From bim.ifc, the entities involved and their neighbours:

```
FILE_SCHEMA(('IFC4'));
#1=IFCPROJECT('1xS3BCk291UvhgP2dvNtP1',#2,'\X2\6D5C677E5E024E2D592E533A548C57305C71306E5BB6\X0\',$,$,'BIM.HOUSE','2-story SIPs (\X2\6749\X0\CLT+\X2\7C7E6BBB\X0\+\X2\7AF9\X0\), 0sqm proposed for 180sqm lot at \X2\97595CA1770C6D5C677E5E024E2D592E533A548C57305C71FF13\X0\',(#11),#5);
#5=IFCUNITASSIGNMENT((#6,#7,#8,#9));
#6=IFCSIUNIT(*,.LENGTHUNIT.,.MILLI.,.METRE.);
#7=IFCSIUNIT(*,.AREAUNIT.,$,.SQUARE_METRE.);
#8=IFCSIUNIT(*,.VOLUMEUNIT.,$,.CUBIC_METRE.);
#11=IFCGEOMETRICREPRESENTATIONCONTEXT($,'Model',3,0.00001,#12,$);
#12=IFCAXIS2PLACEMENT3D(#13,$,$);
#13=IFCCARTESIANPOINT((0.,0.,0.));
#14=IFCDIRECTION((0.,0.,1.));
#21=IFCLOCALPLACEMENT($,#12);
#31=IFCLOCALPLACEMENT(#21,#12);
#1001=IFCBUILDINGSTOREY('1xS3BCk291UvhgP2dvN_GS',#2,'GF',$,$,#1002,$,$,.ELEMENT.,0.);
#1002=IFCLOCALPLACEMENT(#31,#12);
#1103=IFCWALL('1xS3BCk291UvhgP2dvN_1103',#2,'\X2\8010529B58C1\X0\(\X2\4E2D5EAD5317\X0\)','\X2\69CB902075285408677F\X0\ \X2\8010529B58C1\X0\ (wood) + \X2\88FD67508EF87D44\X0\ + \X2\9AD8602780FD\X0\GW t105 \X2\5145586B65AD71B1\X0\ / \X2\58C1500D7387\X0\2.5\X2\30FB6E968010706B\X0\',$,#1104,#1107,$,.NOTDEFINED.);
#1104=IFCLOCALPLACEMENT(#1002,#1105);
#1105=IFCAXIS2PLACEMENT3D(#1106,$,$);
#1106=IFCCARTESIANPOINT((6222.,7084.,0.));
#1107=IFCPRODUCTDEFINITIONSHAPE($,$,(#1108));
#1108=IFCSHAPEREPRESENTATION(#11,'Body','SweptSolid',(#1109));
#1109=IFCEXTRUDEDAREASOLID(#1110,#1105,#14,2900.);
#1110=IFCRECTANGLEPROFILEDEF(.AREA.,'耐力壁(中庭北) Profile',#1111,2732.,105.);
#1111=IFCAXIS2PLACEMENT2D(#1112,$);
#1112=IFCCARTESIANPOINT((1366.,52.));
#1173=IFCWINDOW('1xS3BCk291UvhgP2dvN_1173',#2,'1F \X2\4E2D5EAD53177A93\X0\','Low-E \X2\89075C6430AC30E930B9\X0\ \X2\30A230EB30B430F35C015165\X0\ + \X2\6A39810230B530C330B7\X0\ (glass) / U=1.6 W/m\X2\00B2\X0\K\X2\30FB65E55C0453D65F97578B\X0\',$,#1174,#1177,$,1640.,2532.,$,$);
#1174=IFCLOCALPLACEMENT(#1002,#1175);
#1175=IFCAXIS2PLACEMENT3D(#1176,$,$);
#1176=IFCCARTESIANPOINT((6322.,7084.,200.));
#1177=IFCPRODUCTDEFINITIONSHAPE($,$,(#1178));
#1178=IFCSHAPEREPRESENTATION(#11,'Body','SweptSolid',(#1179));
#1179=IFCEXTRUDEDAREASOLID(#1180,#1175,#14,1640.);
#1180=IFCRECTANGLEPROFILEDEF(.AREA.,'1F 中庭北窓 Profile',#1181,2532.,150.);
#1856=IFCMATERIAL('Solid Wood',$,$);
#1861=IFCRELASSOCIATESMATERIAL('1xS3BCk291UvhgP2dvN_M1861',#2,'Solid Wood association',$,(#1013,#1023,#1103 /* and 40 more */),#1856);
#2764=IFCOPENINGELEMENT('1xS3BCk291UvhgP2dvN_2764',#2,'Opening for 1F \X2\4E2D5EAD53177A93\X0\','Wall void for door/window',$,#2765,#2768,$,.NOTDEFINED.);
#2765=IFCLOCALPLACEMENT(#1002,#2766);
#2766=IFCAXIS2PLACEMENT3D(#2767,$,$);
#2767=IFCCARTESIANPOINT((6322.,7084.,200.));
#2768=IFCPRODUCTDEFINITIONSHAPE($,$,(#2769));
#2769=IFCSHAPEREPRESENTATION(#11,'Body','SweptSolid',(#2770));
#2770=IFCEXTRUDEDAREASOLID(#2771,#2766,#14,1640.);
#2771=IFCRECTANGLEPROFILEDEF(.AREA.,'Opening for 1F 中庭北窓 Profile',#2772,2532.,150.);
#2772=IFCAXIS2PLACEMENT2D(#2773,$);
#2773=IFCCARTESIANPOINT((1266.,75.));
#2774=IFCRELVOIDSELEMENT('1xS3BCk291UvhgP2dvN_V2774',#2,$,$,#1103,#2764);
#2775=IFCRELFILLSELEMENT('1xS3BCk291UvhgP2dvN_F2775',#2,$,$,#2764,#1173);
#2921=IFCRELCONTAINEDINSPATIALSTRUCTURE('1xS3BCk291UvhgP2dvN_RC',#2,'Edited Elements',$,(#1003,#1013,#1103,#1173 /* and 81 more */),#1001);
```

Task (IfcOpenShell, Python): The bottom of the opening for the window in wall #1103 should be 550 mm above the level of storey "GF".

```python
import numpy as np
import ifcopenshell
import ifcopenshell.api.geometry
import ifcopenshell.geom
import ifcopenshell.util.element
import ifcopenshell.util.placement
import ifcopenshell.util.shape
import ifcopenshell.util.unit

model = ifcopenshell.open("bim.ifc")
unit_scale = ifcopenshell.util.unit.calculate_unit_scale(model)

window = model.by_id(1173)
opening = window.FillsVoids[0].RelatingOpeningElement
storey = ifcopenshell.util.element.get_container(window, ifc_class="IfcBuildingStorey")
level = ifcopenshell.util.placement.get_local_placement(storey.ObjectPlacement)[2, 3]

# The opening's origin need not be at the sill, so measure its lowest point.
shape = ifcopenshell.geom.create_shape(ifcopenshell.geom.settings(), opening)
bottom = ifcopenshell.util.shape.get_shape_bottom_elevation(shape, shape.geometry) / unit_scale
dz = level + 0.55 / unit_scale - bottom

shift = np.array([0.0, 0.0, dz])
# The window is not placed relative to its opening, so move both.
for product in (opening, window):
    matrix = ifcopenshell.util.placement.get_local_placement(product.ObjectPlacement)
    matrix[:3, 3] += shift
    ifcopenshell.api.geometry.edit_object_placement(model, product=product, matrix=matrix, is_si=False)

print(f"moved by {dz * unit_scale:+.3f} m")

model.write("bim-out.ifc")
```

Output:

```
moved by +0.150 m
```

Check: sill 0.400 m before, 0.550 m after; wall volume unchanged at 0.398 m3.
